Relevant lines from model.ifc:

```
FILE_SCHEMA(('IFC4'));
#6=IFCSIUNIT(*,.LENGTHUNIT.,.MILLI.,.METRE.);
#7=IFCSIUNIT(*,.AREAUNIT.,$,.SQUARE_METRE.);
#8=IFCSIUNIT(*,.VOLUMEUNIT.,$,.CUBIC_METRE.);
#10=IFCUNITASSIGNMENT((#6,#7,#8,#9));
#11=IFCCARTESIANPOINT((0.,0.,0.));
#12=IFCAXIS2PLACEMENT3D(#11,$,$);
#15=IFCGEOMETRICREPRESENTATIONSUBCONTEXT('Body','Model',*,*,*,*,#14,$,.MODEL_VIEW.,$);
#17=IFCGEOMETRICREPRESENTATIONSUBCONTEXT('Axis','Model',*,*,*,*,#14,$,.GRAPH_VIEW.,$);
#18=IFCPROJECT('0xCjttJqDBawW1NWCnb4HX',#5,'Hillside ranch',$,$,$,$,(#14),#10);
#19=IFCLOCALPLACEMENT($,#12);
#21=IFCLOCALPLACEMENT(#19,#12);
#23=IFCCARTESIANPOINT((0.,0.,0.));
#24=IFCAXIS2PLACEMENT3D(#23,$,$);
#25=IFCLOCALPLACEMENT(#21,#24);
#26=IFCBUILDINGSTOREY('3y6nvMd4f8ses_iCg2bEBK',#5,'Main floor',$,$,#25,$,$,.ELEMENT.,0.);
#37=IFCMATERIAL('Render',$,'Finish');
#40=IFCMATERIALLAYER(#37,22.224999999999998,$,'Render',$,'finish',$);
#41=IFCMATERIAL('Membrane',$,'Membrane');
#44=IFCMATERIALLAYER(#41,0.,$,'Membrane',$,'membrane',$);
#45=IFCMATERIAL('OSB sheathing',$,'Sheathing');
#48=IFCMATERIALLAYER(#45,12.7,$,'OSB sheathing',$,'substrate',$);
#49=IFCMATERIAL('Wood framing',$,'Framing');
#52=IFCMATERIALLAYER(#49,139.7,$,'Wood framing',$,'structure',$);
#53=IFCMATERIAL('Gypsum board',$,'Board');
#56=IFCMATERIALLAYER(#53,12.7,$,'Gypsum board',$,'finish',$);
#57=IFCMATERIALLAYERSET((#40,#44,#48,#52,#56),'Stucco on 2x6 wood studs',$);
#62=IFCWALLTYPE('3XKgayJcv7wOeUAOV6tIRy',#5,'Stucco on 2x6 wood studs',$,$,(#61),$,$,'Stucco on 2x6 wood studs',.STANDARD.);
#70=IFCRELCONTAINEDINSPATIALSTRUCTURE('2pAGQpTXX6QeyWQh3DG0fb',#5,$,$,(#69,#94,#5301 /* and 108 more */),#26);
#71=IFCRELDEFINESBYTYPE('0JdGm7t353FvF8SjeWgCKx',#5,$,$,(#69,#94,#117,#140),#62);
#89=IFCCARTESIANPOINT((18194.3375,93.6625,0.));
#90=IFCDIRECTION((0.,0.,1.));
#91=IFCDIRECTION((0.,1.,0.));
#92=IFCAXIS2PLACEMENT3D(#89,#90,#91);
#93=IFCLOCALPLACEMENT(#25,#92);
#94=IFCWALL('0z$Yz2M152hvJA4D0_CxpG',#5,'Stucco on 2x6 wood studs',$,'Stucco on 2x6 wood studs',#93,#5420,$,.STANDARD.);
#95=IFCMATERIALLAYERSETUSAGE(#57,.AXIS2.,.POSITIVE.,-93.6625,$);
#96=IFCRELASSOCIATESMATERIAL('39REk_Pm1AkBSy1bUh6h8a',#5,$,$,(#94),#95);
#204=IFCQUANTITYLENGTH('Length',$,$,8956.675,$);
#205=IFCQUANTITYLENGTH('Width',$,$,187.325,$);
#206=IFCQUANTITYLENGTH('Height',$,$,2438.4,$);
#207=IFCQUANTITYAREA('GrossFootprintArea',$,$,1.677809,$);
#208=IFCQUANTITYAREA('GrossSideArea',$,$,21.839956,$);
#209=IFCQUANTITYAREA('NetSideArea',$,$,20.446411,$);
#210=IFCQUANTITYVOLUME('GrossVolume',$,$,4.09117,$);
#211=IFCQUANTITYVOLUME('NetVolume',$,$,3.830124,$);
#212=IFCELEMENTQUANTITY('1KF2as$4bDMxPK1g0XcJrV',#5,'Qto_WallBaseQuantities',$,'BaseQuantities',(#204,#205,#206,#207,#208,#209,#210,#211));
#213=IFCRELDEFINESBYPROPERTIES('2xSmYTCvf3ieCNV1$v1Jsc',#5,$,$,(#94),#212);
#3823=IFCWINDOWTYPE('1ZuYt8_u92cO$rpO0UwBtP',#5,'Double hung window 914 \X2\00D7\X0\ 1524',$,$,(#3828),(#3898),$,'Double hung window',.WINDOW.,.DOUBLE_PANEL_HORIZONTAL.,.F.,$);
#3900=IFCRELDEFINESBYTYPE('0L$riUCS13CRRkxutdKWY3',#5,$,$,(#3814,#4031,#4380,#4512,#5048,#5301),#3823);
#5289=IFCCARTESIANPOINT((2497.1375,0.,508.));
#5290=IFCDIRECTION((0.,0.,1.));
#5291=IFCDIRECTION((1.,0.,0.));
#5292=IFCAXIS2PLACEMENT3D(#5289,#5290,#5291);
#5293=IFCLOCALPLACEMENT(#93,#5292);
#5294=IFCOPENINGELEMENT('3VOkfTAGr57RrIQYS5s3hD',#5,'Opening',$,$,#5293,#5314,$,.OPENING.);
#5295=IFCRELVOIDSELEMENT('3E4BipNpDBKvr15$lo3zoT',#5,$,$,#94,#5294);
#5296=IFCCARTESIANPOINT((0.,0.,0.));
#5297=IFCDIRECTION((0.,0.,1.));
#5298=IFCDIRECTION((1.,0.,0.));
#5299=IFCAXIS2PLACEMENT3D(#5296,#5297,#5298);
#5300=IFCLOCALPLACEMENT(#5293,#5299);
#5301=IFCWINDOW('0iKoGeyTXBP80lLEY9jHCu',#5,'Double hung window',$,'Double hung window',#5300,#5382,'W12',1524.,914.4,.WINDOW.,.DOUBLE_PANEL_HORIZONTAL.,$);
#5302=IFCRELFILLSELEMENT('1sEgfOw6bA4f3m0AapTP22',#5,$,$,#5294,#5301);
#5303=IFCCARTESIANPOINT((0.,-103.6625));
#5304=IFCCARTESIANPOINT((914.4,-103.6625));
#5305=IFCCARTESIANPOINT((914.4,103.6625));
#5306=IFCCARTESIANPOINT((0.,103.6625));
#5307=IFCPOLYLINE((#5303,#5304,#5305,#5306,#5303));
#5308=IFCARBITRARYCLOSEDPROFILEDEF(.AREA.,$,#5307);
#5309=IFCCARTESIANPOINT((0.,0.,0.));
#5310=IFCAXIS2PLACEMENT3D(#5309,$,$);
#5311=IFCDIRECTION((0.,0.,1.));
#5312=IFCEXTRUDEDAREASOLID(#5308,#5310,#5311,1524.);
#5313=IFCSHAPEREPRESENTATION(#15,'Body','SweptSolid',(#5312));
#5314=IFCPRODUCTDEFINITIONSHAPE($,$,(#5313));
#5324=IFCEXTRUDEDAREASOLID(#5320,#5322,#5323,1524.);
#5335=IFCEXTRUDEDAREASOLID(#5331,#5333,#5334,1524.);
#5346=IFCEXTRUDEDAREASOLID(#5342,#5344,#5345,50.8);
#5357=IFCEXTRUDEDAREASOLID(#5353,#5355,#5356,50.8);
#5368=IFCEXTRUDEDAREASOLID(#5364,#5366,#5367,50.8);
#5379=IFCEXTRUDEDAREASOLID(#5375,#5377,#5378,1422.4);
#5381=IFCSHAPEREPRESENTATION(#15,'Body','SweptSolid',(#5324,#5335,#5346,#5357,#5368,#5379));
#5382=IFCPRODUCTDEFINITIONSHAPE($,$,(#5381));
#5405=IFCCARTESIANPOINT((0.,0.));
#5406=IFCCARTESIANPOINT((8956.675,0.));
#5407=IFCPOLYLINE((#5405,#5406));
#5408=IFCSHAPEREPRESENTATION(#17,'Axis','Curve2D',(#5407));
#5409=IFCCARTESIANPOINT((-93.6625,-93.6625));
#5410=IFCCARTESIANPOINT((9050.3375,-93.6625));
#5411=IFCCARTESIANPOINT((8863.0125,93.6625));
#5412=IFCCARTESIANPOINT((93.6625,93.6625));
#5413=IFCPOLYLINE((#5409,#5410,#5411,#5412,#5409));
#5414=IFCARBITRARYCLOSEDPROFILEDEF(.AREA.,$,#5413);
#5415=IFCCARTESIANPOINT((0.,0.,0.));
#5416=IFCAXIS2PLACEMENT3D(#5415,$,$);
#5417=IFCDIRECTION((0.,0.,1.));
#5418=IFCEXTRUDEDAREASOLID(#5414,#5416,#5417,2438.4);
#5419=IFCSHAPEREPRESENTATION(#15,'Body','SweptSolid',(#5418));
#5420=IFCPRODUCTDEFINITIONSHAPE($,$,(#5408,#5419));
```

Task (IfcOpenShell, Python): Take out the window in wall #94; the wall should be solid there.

```python
import ifcopenshell
import ifcopenshell.api.feature
import ifcopenshell.api.pset
import ifcopenshell.api.root
import ifcopenshell.geom
import ifcopenshell.util.element
import ifcopenshell.util.shape
import ifcopenshell.util.unit

model = ifcopenshell.open("model.ifc")
area_scale = ifcopenshell.util.unit.calculate_unit_scale(model, "AREAUNIT")
volume_scale = ifcopenshell.util.unit.calculate_unit_scale(model, "VOLUMEUNIT")
settings = ifcopenshell.geom.settings()


def volume(element):
    """Net volume in cubic metres, openings subtracted."""
    shape = ifcopenshell.geom.create_shape(settings, element)
    return ifcopenshell.util.shape.get_volume(shape.geometry)


window = model.by_guid("0iKoGeyTXBP80lLEY9jHCu")
opening = window.FillsVoids[0].RelatingOpeningElement
wall = opening.VoidsElements[0].RelatingBuildingElement
before = volume(wall)

ifcopenshell.api.root.remove_product(model, product=window)
ifcopenshell.api.feature.remove_feature(model, feature=opening)

after = volume(wall)
thickness = 0.1873  # wall thickness in metres

# Update the wall's stored quantities.
qto = model.by_id(ifcopenshell.util.element.get_pset(wall, "Qto_WallBaseQuantities", should_inherit=False)["id"])
ifcopenshell.api.pset.edit_qto(model, qto=qto, properties={
    "NetSideArea": after / thickness / area_scale,
    "NetVolume": after / volume_scale,
})

print(f"wall volume {before:.3f} -> {after:.3f} m3")

model.write("model_edited.ifc")
```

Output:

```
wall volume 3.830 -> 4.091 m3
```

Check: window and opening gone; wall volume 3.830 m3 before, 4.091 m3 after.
